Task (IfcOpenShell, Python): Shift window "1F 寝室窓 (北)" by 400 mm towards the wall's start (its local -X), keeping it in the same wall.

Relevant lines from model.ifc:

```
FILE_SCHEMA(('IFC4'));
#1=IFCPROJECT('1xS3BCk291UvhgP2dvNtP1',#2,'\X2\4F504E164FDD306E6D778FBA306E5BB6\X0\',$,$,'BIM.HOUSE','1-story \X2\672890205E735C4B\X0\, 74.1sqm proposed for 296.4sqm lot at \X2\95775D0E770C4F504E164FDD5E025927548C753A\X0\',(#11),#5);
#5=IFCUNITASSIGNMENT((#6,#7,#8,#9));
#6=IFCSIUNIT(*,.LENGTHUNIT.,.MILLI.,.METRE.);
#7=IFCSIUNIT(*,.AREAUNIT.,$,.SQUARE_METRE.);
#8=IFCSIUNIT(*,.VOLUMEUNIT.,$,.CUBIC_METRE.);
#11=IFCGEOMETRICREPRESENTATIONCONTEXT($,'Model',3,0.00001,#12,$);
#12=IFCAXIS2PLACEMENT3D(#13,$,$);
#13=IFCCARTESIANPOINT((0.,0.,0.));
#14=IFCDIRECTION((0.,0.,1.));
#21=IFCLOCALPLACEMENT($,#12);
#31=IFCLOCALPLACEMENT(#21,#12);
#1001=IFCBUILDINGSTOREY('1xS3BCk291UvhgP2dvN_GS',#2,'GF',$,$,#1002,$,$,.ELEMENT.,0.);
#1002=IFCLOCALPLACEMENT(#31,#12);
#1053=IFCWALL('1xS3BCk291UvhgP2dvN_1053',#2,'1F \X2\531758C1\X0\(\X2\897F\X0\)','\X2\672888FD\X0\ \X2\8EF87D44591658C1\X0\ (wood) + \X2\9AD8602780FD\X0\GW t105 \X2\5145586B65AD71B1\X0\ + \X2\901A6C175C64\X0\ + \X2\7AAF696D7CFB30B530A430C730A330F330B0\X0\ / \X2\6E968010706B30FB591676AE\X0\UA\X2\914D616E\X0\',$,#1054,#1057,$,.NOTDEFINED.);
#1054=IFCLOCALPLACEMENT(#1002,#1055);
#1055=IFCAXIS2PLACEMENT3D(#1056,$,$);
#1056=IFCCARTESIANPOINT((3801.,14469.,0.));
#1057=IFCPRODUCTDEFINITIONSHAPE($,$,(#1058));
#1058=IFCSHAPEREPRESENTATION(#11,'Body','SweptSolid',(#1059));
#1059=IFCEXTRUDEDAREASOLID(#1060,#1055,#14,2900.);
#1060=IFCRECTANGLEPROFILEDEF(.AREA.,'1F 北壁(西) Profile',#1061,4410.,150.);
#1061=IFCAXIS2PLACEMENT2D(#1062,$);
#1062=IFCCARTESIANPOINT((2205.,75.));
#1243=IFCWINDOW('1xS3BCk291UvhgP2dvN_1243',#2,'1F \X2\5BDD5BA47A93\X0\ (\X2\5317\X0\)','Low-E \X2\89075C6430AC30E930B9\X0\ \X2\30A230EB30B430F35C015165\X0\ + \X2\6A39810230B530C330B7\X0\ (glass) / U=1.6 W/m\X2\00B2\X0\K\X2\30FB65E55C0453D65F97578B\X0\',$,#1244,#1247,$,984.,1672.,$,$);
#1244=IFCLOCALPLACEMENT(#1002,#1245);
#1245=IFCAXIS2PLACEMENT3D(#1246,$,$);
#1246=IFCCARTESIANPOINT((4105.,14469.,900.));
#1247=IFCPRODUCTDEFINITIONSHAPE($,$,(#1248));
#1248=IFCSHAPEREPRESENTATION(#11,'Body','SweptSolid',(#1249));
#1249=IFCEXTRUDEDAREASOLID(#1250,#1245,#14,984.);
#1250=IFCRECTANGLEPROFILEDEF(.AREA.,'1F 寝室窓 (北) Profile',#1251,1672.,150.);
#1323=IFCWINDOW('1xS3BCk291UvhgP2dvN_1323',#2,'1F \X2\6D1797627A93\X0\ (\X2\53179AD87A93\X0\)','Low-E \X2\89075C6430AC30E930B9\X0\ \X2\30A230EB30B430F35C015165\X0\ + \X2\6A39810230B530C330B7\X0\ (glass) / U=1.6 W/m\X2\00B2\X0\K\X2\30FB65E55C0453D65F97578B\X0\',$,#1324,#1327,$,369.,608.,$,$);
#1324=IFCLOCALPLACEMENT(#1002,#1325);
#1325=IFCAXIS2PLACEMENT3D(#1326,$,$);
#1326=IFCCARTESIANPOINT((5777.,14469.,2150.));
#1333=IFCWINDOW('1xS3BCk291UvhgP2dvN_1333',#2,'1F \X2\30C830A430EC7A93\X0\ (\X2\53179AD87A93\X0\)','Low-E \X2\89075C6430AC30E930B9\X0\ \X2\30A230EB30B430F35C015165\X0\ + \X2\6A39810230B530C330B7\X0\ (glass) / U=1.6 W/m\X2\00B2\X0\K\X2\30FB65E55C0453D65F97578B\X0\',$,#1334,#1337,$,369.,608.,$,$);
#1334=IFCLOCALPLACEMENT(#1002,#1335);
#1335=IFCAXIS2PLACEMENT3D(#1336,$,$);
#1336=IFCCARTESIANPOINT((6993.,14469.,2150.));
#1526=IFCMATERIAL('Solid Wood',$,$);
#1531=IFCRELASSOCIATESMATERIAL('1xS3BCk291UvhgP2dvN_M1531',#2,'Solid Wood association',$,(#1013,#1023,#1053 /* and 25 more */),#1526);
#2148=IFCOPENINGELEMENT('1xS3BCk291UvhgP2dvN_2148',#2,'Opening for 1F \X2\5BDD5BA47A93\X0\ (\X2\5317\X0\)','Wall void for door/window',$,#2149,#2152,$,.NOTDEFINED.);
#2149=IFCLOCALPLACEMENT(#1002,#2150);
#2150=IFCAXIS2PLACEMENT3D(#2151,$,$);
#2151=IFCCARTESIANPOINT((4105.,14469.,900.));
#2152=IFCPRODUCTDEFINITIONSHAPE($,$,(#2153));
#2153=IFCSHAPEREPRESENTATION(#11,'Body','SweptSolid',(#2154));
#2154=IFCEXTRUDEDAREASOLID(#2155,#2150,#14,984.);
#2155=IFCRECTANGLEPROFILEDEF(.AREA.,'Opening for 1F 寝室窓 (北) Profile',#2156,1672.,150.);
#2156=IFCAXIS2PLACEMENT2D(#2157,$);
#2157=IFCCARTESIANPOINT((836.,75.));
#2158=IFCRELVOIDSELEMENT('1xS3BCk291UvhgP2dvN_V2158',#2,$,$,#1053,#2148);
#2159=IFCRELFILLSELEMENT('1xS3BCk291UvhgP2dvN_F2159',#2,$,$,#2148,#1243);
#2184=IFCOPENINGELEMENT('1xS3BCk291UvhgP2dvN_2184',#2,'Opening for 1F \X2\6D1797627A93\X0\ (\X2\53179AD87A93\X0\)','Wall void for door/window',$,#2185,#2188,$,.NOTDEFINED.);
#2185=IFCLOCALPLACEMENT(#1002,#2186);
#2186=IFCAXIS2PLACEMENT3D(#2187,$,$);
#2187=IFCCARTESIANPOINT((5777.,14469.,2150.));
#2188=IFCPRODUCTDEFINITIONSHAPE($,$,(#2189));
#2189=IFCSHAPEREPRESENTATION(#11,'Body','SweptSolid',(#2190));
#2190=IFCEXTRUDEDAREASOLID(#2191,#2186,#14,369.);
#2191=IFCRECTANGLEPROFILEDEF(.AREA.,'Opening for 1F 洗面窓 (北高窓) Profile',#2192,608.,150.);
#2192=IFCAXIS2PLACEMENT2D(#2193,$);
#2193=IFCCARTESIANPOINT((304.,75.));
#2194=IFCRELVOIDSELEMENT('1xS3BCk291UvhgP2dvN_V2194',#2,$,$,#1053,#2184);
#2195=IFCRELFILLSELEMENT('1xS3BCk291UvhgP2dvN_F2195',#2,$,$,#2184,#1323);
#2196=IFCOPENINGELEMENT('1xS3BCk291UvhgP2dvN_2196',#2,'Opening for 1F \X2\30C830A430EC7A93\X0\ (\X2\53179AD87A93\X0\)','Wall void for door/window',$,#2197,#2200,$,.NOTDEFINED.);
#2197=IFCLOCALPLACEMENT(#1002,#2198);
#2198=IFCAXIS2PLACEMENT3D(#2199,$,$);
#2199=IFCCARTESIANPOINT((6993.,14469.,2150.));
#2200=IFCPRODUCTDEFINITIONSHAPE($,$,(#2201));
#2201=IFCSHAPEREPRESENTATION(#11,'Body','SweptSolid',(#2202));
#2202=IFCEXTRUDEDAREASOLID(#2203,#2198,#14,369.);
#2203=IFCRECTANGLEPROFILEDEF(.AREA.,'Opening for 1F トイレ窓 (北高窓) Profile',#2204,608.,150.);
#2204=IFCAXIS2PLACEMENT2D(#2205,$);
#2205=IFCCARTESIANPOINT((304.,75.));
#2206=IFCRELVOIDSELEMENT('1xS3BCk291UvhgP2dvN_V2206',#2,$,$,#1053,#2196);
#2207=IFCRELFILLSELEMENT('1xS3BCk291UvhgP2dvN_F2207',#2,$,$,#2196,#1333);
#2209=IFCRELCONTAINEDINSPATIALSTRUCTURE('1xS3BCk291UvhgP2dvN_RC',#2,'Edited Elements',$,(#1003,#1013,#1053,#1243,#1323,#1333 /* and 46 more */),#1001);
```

```python
import ifcopenshell
import ifcopenshell.api.geometry
import ifcopenshell.util.placement

model = ifcopenshell.open("model.ifc")

window = model.by_guid("1xS3BCk291UvhgP2dvN_1243")
opening = window.FillsVoids[0].RelatingOpeningElement
wall = opening.VoidsElements[0].RelatingBuildingElement

wall_matrix = ifcopenshell.util.placement.get_local_placement(wall.ObjectPlacement)
shift = wall_matrix[:3, 0] * -400.0
before = ifcopenshell.util.placement.get_local_placement(window.ObjectPlacement)[:3, 3].copy()

# The window is not placed relative to its opening, so move both.
for product in (opening, window):
    matrix = ifcopenshell.util.placement.get_local_placement(product.ObjectPlacement)
    matrix[:3, 3] += shift
    ifcopenshell.api.geometry.edit_object_placement(model, product=product, matrix=matrix, is_si=False)

after = ifcopenshell.util.placement.get_local_placement(window.ObjectPlacement)[:3, 3]
print("window moved by", (after - before).round(3) + 0.0)

model.write("model-out.ifc")
```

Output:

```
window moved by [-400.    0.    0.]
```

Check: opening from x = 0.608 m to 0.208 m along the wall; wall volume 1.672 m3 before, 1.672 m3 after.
